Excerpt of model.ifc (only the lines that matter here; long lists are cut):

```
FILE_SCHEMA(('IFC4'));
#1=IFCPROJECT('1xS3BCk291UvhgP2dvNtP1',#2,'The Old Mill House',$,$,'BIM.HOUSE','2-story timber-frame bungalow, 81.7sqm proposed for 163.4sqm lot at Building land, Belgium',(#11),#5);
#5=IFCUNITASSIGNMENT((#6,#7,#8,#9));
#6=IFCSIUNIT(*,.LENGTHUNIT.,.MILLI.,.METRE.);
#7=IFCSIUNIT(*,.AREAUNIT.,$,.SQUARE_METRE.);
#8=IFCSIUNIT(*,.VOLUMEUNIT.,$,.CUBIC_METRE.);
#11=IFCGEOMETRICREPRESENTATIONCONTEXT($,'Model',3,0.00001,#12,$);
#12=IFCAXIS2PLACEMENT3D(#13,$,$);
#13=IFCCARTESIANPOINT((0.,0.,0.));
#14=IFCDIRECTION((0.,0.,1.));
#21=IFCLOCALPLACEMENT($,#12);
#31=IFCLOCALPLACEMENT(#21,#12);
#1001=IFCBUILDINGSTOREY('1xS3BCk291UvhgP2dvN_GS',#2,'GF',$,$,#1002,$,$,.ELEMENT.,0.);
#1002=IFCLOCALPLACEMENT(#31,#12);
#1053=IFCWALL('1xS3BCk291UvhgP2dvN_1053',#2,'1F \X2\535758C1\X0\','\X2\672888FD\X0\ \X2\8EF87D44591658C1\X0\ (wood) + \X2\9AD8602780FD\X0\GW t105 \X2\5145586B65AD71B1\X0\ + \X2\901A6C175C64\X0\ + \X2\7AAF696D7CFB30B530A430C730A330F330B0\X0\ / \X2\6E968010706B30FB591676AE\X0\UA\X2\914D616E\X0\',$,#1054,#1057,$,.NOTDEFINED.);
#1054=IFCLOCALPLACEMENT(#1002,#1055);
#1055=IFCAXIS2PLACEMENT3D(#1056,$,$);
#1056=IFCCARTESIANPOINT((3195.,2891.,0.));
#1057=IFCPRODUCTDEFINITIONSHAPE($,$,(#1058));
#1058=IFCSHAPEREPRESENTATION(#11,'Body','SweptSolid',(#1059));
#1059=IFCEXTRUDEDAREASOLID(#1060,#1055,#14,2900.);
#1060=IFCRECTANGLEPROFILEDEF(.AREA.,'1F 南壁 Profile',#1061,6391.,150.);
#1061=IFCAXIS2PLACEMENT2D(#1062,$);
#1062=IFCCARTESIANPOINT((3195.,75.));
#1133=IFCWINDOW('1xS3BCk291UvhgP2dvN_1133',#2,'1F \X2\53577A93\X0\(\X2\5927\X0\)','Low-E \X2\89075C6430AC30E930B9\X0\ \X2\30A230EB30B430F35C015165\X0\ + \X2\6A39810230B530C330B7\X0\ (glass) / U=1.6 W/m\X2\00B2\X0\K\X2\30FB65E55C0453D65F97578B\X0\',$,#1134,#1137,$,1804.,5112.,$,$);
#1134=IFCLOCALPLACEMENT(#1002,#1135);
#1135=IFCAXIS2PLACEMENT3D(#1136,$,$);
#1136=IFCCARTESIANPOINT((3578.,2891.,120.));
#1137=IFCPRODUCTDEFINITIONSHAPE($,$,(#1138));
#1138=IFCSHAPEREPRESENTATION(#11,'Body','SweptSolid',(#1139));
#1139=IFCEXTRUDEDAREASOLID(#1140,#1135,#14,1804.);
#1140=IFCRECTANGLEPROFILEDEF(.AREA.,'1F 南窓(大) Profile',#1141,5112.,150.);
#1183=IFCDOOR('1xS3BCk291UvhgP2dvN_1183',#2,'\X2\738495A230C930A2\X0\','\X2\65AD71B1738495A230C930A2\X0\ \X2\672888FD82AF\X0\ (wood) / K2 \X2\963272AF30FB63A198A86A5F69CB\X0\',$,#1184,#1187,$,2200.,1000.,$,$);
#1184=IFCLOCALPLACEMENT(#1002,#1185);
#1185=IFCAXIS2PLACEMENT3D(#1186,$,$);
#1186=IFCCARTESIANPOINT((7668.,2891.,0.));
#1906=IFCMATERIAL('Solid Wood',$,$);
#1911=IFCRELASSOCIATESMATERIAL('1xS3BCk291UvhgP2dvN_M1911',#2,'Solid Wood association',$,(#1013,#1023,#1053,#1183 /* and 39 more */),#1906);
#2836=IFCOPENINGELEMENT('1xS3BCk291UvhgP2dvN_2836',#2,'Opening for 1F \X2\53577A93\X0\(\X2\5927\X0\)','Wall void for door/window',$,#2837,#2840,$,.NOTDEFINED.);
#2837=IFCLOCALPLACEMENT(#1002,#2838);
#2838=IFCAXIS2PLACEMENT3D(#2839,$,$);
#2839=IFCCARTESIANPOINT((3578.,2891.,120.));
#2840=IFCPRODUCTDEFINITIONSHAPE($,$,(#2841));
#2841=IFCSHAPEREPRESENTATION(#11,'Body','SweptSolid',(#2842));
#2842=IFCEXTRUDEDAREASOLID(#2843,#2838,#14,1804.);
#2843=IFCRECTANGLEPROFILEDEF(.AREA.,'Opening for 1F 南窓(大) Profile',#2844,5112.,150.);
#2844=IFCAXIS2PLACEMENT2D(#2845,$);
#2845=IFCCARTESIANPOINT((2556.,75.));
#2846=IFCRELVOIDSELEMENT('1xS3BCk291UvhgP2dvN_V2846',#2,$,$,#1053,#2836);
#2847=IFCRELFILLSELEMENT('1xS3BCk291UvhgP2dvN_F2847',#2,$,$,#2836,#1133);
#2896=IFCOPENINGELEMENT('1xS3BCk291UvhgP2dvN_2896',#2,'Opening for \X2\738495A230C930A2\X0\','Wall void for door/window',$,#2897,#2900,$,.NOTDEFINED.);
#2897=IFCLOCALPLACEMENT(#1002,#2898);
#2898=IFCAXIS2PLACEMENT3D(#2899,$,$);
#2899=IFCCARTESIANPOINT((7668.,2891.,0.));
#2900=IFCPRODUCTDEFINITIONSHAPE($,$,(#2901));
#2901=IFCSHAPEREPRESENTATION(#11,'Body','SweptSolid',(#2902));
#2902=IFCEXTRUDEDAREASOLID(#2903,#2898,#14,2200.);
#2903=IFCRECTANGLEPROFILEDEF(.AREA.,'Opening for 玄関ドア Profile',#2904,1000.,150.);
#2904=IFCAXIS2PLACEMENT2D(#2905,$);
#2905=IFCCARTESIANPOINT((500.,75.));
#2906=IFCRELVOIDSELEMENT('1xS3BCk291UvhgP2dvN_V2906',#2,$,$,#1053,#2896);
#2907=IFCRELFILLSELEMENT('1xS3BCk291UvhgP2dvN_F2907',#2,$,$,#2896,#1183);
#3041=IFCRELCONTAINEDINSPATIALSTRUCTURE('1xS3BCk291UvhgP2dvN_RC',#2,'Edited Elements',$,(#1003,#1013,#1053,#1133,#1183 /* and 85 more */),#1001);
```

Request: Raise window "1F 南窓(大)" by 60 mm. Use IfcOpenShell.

```python
import numpy as np
import ifcopenshell
import ifcopenshell.api.geometry
import ifcopenshell.util.placement
import ifcopenshell.util.unit

model = ifcopenshell.open("model.ifc")
unit_scale = ifcopenshell.util.unit.calculate_unit_scale(model)

window = model.by_guid("1xS3BCk291UvhgP2dvN_1133")
opening = window.FillsVoids[0].RelatingOpeningElement
dz = 60.0

shift = np.array([0.0, 0.0, dz])
# The window is not placed relative to its opening, so move both.
for product in (opening, window):
    matrix = ifcopenshell.util.placement.get_local_placement(product.ObjectPlacement)
    matrix[:3, 3] += shift
    ifcopenshell.api.geometry.edit_object_placement(model, product=product, matrix=matrix, is_si=False)

print(f"moved by {dz * unit_scale:+.3f} m")

model.write("model_v2.ifc")
```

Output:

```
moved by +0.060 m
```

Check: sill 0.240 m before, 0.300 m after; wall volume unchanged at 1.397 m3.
